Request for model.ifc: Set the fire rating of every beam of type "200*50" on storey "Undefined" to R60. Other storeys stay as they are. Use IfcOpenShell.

First a look at what the model holds.

```python
import ifcopenshell
import ifcopenshell.util.element

model = ifcopenshell.open("model.ifc")
print(model.schema)
storey = next(s for s in model.by_type("IfcBuildingStorey") if s.Name == "Undefined")
beams = [e for e in ifcopenshell.util.element.get_decomposition(storey) if e.is_a("IfcBeam")]
seen = {}
for e in beams:
    element_type = ifcopenshell.util.element.get_type(e)
    key = (element_type.Name if element_type != e and element_type else None, ifcopenshell.util.element.get_pset(e, "Pset_BeamCommon", "FireRating"))
    seen[key] = seen.get(key, 0) + 1
for (name, value), count in sorted(seen.items(), key=str):
    print(count, "x", name, "|", value)
```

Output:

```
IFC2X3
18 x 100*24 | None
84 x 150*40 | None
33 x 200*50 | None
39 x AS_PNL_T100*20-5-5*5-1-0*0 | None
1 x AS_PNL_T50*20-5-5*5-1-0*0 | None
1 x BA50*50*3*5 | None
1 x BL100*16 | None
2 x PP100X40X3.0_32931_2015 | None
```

```python
import ifcopenshell
import ifcopenshell.api.pset
import ifcopenshell.util.element

model = ifcopenshell.open("model.ifc")

storey = next(s for s in model.by_type("IfcBuildingStorey") if s.Name == "Undefined")
beams = [e for e in ifcopenshell.util.element.get_decomposition(storey) if e.is_a("IfcBeam")]

count = 0
for e in beams:
    element_type = ifcopenshell.util.element.get_type(e)
    if element_type in (None, e) or element_type.Name != "200*50":
        continue
    found = ifcopenshell.util.element.get_pset(e, "Pset_BeamCommon", should_inherit=False)
    if found:
        pset = model.by_id(found["id"])
        if len(ifcopenshell.util.element.get_elements_by_pset(pset)) > 1:
            pset = ifcopenshell.api.pset.unshare_pset(model, products=[e], pset=pset)[0]
    else:
        pset = ifcopenshell.api.pset.add_pset(model, product=e, name="Pset_BeamCommon")
    ifcopenshell.api.pset.edit_pset(model, pset=pset, properties={"FireRating": "R60"})
    count += 1

print(count, "beams updated")

model.write("model-out.ifc")
```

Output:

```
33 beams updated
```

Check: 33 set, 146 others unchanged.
